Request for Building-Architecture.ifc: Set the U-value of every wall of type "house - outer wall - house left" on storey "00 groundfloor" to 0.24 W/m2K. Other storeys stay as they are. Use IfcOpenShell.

First a look at what the model holds.

```python
import ifcopenshell
import ifcopenshell.util.element

model = ifcopenshell.open("Building-Architecture.ifc")
print(model.schema)
storey = next(s for s in model.by_type("IfcBuildingStorey") if s.Name == "00 groundfloor")
walls = [e for e in ifcopenshell.util.element.get_decomposition(storey) if e.is_a("IfcWall")]
seen = {}
for e in walls:
    element_type = ifcopenshell.util.element.get_type(e)
    key = (element_type.Name if element_type != e and element_type else None, ifcopenshell.util.element.get_pset(e, "Pset_WallCommon", "ThermalTransmittance"))
    seen[key] = seen.get(key, 0) + 1
for (name, value), count in sorted(seen.items(), key=str):
    print(count, "x", name, "|", value)
```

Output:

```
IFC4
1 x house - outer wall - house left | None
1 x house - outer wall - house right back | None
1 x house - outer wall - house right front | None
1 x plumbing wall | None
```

```python
import ifcopenshell
import ifcopenshell.api.pset
import ifcopenshell.util.element

model = ifcopenshell.open("Building-Architecture.ifc")

storey = next(s for s in model.by_type("IfcBuildingStorey") if s.Name == "00 groundfloor")
walls = [e for e in ifcopenshell.util.element.get_decomposition(storey) if e.is_a("IfcWall")]

count = 0
for e in walls:
    element_type = ifcopenshell.util.element.get_type(e)
    if element_type in (None, e) or element_type.Name != "house - outer wall - house left":
        continue
    # add_pset returns the element's existing set when there is one.
    pset = ifcopenshell.api.pset.add_pset(model, product=e, name="Pset_WallCommon")
    ifcopenshell.api.pset.edit_pset(model, pset=pset, properties={"ThermalTransmittance": 0.24})
    count += 1

print(count, "walls updated")

model.write("Building-Architecture-out.ifc")
```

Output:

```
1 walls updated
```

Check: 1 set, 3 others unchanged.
